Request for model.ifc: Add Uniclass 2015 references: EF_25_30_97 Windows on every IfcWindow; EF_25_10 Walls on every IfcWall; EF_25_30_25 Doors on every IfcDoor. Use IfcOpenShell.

First a look at what the model holds.

```python
import ifcopenshell

model = ifcopenshell.open("model.ifc")
print(model.schema)
print("classifications:", [c.Name for c in model.by_type("IfcClassification")])
for ifc_class in ("IfcDoor", "IfcRoof", "IfcStair", "IfcWall", "IfcWindow"):
    print(ifc_class, len(model.by_type(ifc_class)))
```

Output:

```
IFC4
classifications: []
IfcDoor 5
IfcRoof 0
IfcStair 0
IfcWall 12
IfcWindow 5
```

```python
import ifcopenshell
import ifcopenshell.api.classification

model = ifcopenshell.open("model.ifc")

system = ifcopenshell.api.classification.add_classification(model, classification="Uniclass 2015")

codes = {
    "IfcWindow": ("EF_25_30_97", "Windows"),
    "IfcWall": ("EF_25_10", "Walls"),
    "IfcDoor": ("EF_25_30_25", "Doors"),
}
for ifc_class, (code, name) in codes.items():
    products = model.by_type(ifc_class)
    ifcopenshell.api.classification.add_reference(
        model, products=products, classification=system, identification=code, name=name
    )
    print(code, len(products))

model.write("model_v2.ifc")
```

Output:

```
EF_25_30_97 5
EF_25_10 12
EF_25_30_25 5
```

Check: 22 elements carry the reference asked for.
